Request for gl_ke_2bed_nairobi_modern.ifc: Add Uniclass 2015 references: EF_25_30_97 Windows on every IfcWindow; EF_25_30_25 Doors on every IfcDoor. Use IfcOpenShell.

First a look at what the model holds.

```python
import ifcopenshell

model = ifcopenshell.open("gl_ke_2bed_nairobi_modern.ifc")
print(model.schema)
print("classifications:", [c.Name for c in model.by_type("IfcClassification")])
for ifc_class in ("IfcDoor", "IfcRoof", "IfcStair", "IfcWall", "IfcWindow"):
    print(ifc_class, len(model.by_type(ifc_class)))
```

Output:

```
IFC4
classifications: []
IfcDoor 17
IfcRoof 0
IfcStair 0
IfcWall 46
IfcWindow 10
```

```python
import ifcopenshell
import ifcopenshell.api.classification

model = ifcopenshell.open("gl_ke_2bed_nairobi_modern.ifc")

system = ifcopenshell.api.classification.add_classification(model, classification="Uniclass 2015")

codes = {
    "IfcWindow": ("EF_25_30_97", "Windows"),
    "IfcDoor": ("EF_25_30_25", "Doors"),
}
for ifc_class, (code, name) in codes.items():
    products = model.by_type(ifc_class)
    ifcopenshell.api.classification.add_reference(
        model, products=products, classification=system, identification=code, name=name
    )
    print(code, len(products))

model.write("gl_ke_2bed_nairobi_modern_rev.ifc")
```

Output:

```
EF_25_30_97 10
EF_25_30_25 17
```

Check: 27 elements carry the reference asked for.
